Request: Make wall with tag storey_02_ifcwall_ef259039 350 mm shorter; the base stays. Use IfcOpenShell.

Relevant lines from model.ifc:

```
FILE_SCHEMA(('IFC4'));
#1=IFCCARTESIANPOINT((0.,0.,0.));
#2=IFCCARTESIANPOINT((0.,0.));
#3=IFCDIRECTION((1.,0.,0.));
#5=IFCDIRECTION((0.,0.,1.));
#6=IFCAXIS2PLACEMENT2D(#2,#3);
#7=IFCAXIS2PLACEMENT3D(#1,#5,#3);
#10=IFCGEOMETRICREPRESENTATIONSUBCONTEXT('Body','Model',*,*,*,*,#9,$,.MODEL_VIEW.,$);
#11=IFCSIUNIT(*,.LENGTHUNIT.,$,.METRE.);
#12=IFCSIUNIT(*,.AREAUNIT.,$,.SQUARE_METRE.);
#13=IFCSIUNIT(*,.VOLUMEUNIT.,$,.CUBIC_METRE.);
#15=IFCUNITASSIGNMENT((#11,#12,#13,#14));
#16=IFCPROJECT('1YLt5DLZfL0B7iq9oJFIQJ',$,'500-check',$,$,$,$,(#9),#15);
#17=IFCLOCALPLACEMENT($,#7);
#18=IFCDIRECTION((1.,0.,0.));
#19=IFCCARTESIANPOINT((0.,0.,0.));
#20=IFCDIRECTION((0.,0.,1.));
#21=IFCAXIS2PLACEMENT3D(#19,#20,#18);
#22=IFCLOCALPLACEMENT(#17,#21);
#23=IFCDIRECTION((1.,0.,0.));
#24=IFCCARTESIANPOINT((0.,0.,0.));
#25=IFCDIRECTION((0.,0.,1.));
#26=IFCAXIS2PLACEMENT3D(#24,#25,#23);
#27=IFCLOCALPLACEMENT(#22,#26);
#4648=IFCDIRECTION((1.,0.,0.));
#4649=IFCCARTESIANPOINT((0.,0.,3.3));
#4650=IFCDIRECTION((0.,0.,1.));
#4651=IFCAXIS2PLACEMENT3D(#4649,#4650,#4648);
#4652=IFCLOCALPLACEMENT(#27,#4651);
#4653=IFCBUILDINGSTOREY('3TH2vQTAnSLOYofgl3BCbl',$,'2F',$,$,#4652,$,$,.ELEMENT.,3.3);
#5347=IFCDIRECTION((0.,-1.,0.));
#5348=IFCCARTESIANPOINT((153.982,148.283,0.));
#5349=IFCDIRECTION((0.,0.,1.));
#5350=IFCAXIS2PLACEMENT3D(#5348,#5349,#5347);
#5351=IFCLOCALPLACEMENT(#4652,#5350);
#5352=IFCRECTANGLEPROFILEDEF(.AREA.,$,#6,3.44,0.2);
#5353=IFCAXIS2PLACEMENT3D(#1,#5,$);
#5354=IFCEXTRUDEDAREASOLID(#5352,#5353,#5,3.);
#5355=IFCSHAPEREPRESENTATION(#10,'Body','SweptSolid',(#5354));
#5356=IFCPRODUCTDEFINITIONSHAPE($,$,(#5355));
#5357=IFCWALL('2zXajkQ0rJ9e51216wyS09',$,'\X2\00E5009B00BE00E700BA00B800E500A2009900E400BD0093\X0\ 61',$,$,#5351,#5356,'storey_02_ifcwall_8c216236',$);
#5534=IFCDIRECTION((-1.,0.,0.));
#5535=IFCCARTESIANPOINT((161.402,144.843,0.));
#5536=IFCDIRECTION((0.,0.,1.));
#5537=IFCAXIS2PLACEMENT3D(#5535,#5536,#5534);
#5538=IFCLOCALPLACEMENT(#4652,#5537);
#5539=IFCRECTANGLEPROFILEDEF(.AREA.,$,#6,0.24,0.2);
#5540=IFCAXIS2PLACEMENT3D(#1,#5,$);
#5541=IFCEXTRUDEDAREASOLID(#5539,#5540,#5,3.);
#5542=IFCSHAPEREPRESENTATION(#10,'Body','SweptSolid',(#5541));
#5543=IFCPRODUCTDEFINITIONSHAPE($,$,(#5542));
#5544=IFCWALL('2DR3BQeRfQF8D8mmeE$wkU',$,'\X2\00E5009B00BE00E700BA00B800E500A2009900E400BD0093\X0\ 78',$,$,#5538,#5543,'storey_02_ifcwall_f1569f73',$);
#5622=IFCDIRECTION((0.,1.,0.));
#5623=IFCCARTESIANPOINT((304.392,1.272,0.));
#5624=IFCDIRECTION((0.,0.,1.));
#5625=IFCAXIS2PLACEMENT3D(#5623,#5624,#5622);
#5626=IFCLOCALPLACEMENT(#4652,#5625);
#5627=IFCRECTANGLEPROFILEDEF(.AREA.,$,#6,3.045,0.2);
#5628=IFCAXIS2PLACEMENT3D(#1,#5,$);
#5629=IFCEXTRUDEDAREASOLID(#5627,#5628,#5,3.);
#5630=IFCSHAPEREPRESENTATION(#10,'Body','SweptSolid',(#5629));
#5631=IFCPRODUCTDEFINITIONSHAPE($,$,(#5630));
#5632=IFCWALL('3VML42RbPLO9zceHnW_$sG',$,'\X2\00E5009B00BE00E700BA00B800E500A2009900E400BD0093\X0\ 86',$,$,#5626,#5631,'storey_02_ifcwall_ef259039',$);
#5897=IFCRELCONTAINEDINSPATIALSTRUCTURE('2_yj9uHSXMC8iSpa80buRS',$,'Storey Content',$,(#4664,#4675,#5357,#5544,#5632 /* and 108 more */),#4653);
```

```python
import ifcopenshell
import ifcopenshell.geom
import ifcopenshell.util.representation
import ifcopenshell.util.shape
import ifcopenshell.util.unit

model = ifcopenshell.open("model.ifc")
unit_scale = ifcopenshell.util.unit.calculate_unit_scale(model)
settings = ifcopenshell.geom.settings()


def volume(element):
    """Net volume in cubic metres, openings subtracted."""
    shape = ifcopenshell.geom.create_shape(settings, element)
    return ifcopenshell.util.shape.get_volume(shape.geometry)


wall = model.by_id(5632)
before = volume(wall)

body = ifcopenshell.util.representation.get_representation(wall, "Model", "Body")
solid = body.Items[0]
old_height = solid.Depth
solid.Depth -= 0.35 / unit_scale
after = volume(wall)

print(f"height {old_height:g} -> {solid.Depth:g}, volume {before:.3f} -> {after:.3f} m3")

model.write("model-out.ifc")
```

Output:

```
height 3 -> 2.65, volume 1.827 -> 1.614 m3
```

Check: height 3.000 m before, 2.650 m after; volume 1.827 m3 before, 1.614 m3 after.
